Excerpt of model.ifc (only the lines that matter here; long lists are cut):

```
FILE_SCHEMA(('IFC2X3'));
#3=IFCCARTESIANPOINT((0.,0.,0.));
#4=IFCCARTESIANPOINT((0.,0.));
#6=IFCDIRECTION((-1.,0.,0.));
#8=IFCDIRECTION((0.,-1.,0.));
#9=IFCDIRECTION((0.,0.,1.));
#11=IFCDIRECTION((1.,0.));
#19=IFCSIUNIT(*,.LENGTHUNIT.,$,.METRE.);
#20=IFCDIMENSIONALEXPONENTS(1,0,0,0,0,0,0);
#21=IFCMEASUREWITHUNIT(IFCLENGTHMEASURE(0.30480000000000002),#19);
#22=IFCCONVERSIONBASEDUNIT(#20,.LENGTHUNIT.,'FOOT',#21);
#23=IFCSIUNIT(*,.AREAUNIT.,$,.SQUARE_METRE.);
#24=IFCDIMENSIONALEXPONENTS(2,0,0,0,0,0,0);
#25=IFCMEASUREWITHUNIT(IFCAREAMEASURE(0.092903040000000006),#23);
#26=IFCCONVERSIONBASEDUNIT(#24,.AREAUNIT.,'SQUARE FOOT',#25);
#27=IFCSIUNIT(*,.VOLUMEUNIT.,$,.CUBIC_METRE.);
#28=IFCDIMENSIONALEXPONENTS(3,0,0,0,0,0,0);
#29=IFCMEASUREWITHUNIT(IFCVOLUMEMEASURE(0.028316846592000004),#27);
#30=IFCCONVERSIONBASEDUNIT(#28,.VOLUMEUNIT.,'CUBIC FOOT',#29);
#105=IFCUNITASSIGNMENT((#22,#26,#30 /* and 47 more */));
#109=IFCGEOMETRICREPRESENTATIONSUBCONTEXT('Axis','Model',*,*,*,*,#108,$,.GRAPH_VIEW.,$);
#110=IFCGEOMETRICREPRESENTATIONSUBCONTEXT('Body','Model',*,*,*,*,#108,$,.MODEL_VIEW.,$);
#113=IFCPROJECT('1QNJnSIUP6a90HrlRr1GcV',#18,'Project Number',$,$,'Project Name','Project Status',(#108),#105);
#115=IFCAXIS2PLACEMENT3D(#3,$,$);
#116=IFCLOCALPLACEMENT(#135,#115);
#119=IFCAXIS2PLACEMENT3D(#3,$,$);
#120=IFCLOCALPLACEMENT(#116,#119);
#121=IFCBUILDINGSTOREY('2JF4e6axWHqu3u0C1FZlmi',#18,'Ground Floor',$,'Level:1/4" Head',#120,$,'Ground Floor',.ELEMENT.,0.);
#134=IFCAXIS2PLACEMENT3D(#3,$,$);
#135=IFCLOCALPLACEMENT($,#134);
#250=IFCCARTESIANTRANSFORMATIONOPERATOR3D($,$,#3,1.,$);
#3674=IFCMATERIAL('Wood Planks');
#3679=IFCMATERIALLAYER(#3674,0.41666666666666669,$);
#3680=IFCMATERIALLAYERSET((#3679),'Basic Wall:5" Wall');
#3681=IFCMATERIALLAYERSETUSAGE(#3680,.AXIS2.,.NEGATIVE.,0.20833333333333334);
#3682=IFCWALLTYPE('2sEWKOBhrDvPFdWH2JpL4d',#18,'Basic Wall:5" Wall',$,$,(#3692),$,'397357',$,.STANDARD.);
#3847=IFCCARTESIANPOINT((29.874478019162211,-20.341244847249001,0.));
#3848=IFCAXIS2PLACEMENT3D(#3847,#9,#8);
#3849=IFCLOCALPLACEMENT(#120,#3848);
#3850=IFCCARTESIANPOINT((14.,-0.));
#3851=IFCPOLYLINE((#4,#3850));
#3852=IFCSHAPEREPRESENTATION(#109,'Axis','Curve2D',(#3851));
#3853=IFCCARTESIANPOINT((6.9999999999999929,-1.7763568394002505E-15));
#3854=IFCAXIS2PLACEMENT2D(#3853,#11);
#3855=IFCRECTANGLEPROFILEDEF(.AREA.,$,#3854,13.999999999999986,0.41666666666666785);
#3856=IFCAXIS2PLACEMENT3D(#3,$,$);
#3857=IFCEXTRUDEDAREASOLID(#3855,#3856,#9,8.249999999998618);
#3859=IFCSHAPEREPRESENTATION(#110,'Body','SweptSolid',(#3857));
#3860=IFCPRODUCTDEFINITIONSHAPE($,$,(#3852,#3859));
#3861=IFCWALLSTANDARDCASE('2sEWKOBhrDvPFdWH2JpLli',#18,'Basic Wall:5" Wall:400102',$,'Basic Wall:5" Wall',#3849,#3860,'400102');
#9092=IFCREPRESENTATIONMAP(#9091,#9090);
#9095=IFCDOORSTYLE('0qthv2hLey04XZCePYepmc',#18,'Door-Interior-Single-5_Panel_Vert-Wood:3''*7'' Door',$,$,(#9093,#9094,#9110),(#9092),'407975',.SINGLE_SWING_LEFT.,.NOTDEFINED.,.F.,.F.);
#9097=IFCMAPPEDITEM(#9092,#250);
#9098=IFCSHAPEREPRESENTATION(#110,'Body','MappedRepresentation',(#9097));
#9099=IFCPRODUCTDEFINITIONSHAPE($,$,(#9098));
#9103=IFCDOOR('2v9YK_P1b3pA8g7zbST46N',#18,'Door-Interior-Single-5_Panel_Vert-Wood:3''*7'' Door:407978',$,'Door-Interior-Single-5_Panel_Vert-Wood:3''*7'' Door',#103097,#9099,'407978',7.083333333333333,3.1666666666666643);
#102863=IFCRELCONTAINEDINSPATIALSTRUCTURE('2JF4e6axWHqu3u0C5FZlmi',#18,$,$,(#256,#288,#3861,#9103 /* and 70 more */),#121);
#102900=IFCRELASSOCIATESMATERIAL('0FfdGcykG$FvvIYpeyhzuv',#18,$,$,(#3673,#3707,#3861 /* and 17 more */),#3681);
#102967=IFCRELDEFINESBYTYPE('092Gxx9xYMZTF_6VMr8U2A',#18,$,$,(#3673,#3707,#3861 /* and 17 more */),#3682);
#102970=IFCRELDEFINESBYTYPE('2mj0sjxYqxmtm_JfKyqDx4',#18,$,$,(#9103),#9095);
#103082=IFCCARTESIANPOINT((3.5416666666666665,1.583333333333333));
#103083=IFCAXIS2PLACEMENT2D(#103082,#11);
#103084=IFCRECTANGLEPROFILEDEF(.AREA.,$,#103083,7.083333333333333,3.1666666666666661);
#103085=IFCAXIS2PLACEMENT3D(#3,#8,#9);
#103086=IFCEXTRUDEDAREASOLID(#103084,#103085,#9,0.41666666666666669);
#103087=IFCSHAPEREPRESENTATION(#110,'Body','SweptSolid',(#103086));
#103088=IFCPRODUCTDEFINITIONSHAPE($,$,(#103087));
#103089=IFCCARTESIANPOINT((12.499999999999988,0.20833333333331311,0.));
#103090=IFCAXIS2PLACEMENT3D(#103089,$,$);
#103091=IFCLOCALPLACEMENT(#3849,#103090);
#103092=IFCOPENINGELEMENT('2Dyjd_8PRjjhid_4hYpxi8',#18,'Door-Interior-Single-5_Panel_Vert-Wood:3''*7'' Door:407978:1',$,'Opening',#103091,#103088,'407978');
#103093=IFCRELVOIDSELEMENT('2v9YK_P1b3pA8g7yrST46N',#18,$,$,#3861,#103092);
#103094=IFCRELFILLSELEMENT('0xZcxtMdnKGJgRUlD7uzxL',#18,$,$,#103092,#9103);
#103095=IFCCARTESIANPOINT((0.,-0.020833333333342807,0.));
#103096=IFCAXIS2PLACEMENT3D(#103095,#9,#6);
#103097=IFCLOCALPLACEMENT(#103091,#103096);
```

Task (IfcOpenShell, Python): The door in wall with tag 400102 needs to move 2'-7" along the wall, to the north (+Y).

```python
import ifcopenshell
import ifcopenshell.api.geometry
import ifcopenshell.util.placement
import ifcopenshell.util.unit

model = ifcopenshell.open("model.ifc")
unit_scale = ifcopenshell.util.unit.calculate_unit_scale(model)

door = model.by_id(9103)
opening = door.FillsVoids[0].RelatingOpeningElement
wall = opening.VoidsElements[0].RelatingBuildingElement

wall_matrix = ifcopenshell.util.placement.get_local_placement(wall.ObjectPlacement)
shift = wall_matrix[:3, 0] * -31 * 0.0254 / unit_scale
before = ifcopenshell.util.placement.get_local_placement(door.ObjectPlacement)[:3, 3].copy()

# The door is placed relative to its opening, so it follows when the opening moves.
matrix = ifcopenshell.util.placement.get_local_placement(opening.ObjectPlacement)
matrix[:3, 3] += shift
ifcopenshell.api.geometry.edit_object_placement(
    model, product=opening, matrix=matrix, is_si=False, should_transform_children=True
)

after = ifcopenshell.util.placement.get_local_placement(door.ObjectPlacement)[:3, 3]
print("door moved by", (after - before).round(3) + 0.0)

model.write("model_rev.ifc")
```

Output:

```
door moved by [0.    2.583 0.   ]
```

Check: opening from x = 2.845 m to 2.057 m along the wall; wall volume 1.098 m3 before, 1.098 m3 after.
